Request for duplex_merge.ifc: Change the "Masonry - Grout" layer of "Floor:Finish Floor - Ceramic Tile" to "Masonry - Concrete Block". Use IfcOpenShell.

First a look at what the model holds.

```python
import ifcopenshell
import ifcopenshell.util.element

model = ifcopenshell.open("duplex_merge.ifc")
print(model.schema)
for layer_set in model.by_type("IfcMaterialLayerSet"):
    if layer_set.LayerSetName == "Floor:Finish Floor - Ceramic Tile":
        for layer in layer_set.MaterialLayers:
            print(layer.id(), layer.Material and layer.Material.Name, layer.LayerThickness, sep=" | ")
        print(len(ifcopenshell.util.element.get_elements_by_material(model, layer_set)), "elements and types use it")
print(sorted(m.Name for m in model.by_type("IfcMaterial") if m.Name)[:60])
```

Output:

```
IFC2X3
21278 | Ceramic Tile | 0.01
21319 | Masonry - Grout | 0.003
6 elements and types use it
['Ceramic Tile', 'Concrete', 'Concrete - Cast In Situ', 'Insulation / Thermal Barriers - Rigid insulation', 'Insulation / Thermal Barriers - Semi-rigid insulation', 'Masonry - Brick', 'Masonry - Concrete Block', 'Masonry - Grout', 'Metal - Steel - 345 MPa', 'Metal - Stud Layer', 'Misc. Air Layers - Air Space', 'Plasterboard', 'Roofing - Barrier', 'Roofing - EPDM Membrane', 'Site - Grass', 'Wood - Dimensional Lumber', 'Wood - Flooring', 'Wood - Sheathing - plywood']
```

```python
import ifcopenshell
import ifcopenshell.api.material

model = ifcopenshell.open("duplex_merge.ifc")

layer_set = next(s for s in model.by_type("IfcMaterialLayerSet") if s.LayerSetName == "Floor:Finish Floor - Ceramic Tile")
layer = next(l for l in layer_set.MaterialLayers if l.Material and l.Material.Name == "Masonry - Grout")
material = next(m for m in model.by_type("IfcMaterial") if m.Name == "Masonry - Concrete Block")

# Point this one layer at the other material; renaming the old one would change it everywhere.
ifcopenshell.api.material.edit_layer(model, layer=layer, attributes={}, material=material)

print([l.Material.Name if l.Material else None for l in layer_set.MaterialLayers])

model.write("duplex_merge-out.ifc")
```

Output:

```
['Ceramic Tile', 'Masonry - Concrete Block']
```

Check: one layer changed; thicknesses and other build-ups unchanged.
